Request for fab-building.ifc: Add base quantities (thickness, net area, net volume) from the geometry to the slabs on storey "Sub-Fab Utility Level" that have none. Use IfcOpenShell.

First a look at what the model holds.

```python
import ifcopenshell
import ifcopenshell.util.element
import ifcopenshell.util.unit

model = ifcopenshell.open("fab-building.ifc")
print(model.schema)
for unit_type in ("LENGTHUNIT", "AREAUNIT", "VOLUMEUNIT"):
    print(unit_type, ifcopenshell.util.unit.calculate_unit_scale(model, unit_type))
storey = next(s for s in model.by_type("IfcBuildingStorey") if s.Name == "Sub-Fab Utility Level")
slabs = [e for e in ifcopenshell.util.element.get_decomposition(storey) if e.is_a("IfcSlab")]
for e in sorted(slabs, key=lambda e: e.id()):
    print(e.id(), e.is_a(), e.Name, list(ifcopenshell.util.element.get_psets(e, qtos_only=True)), sep=" | ")
```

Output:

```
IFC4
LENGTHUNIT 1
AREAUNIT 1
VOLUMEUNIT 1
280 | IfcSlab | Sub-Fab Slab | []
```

```python
import ifcopenshell
import ifcopenshell.api.pset
import ifcopenshell.geom
import ifcopenshell.util.element
import ifcopenshell.util.shape
import ifcopenshell.util.unit

model = ifcopenshell.open("fab-building.ifc")
unit_scale = ifcopenshell.util.unit.calculate_unit_scale(model)
area_scale = ifcopenshell.util.unit.calculate_unit_scale(model, "AREAUNIT")
volume_scale = ifcopenshell.util.unit.calculate_unit_scale(model, "VOLUMEUNIT")
settings = ifcopenshell.geom.settings()

storey = next(s for s in model.by_type("IfcBuildingStorey") if s.Name == "Sub-Fab Utility Level")
slabs = [e for e in ifcopenshell.util.element.get_decomposition(storey) if e.is_a("IfcSlab")]

for e in sorted(slabs, key=lambda e: e.id()):
    if ifcopenshell.util.element.get_psets(e, qtos_only=True, should_inherit=False):
        continue
    # Geometry comes back in metres, in the element's own axes.
    shape = ifcopenshell.geom.create_shape(settings, e)
    values = {
        "Width": ifcopenshell.util.shape.get_z(shape.geometry) / unit_scale,
        "NetArea": ifcopenshell.util.shape.get_footprint_area(shape.geometry) / area_scale,
        "NetVolume": ifcopenshell.util.shape.get_volume(shape.geometry) / volume_scale,
    }
    qto = ifcopenshell.api.pset.add_qto(model, product=e, name="Qto_SlabBaseQuantities")
    ifcopenshell.api.pset.edit_qto(model, qto=qto, properties=values)
    print(e.id(), {k: round(v, 3) for k, v in values.items()})

model.write("fab-building_v2.ifc")
```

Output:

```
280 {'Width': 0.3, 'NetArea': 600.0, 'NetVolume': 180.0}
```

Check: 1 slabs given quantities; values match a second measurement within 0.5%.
